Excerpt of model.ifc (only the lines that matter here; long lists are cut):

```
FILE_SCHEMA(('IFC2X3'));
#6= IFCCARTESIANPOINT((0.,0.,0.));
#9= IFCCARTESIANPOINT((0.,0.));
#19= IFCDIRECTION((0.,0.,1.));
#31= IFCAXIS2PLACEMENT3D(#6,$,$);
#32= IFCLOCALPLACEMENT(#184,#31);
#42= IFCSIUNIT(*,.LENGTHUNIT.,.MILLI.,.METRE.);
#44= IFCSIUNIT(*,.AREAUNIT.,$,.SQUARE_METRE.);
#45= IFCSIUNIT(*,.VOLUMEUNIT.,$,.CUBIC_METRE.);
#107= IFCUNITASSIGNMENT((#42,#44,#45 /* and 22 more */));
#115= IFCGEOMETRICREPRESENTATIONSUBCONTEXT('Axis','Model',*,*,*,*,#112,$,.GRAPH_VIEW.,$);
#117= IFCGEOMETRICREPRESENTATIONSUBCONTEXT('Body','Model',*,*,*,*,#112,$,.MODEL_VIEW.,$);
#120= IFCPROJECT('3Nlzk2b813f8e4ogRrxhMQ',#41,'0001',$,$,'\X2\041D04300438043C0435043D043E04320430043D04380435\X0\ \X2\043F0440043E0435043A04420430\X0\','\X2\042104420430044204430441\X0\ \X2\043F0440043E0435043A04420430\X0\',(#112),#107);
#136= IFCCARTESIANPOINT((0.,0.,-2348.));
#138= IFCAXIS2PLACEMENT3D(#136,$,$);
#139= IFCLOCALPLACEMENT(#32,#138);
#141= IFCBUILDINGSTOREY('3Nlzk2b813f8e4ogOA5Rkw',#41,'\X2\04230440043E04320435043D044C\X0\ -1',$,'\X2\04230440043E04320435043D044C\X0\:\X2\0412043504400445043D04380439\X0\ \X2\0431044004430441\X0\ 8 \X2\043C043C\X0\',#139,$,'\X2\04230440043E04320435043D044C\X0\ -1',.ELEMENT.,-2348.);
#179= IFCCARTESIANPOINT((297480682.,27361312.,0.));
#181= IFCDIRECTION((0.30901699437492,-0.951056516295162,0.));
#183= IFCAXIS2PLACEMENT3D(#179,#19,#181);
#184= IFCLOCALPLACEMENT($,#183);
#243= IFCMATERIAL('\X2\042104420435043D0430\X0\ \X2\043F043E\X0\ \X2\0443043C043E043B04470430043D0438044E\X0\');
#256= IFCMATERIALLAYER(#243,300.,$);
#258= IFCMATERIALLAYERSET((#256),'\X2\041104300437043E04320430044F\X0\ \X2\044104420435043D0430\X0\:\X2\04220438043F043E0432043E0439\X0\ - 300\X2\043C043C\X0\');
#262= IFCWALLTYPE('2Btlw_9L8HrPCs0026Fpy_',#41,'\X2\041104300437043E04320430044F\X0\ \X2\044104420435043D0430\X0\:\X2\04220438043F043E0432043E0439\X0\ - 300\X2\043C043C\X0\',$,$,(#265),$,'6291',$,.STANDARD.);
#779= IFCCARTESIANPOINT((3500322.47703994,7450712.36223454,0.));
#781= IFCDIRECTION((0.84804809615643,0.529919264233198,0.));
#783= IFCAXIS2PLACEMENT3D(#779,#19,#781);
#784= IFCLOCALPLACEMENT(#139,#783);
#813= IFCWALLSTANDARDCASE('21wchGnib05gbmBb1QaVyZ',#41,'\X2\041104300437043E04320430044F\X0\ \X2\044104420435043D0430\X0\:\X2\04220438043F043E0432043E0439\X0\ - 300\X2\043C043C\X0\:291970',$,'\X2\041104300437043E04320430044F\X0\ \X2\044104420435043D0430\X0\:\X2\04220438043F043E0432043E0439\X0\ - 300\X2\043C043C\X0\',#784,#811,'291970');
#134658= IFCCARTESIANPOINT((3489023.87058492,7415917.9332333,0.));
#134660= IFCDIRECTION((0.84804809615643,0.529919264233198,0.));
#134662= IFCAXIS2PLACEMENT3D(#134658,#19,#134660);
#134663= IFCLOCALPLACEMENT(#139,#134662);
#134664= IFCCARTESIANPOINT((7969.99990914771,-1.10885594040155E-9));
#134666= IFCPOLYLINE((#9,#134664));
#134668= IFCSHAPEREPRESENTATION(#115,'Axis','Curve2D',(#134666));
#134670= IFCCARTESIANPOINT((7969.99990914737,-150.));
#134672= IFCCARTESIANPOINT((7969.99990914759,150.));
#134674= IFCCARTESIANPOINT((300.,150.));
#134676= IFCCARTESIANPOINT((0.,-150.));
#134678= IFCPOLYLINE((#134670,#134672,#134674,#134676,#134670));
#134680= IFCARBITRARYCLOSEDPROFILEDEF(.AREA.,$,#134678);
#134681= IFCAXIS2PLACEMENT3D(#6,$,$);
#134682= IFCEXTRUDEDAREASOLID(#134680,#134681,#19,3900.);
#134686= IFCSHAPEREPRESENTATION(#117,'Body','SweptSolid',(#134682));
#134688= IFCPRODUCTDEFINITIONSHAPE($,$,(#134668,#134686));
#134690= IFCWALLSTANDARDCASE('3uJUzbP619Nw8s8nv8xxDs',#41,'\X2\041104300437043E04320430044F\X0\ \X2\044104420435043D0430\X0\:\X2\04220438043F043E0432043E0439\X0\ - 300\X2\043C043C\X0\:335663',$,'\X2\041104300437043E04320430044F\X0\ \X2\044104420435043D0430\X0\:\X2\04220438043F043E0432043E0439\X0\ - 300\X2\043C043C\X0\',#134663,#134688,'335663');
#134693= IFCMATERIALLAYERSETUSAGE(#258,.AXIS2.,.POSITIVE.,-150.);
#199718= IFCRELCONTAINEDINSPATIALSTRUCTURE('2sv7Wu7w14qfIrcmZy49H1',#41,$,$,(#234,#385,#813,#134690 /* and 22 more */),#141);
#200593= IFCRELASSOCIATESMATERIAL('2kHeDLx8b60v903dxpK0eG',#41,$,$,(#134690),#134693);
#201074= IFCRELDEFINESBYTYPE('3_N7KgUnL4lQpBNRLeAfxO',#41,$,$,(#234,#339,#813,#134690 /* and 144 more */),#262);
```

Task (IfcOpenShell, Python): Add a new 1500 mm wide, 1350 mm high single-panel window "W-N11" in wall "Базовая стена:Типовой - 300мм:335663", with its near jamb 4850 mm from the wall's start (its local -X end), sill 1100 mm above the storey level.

```python
import numpy as np
import ifcopenshell
import ifcopenshell.api.feature
import ifcopenshell.api.geometry
import ifcopenshell.api.root
import ifcopenshell.api.spatial
import ifcopenshell.api.type
import ifcopenshell.geom
import ifcopenshell.util.element
import ifcopenshell.util.placement
import ifcopenshell.util.representation
import ifcopenshell.util.shape
import ifcopenshell.util.unit

model = ifcopenshell.open("model.ifc")
unit_scale = ifcopenshell.util.unit.calculate_unit_scale(model)
settings = ifcopenshell.geom.settings()


def volume(element):
    """Net volume in cubic metres, openings subtracted."""
    shape = ifcopenshell.geom.create_shape(settings, element)
    return ifcopenshell.util.shape.get_volume(shape.geometry)


wall = model.by_guid("3uJUzbP619Nw8s8nv8xxDs")
storey = ifcopenshell.util.element.get_container(wall, ifc_class="IfcBuildingStorey")
context = ifcopenshell.util.representation.get_context(model, "Model", "Body", "MODEL_VIEW")
before = volume(wall)

width, height, from_end, sill = 1.5, 1.35, 4.85, 1.1  # metres

# The wall runs along its own X axis, and the end named is its -X end.
wall_shape = ifcopenshell.geom.create_shape(settings, wall)
x, y, z = ifcopenshell.util.shape.get_vertices(wall_shape.geometry).T
start = x.min() + from_end
face, thickness = float(y.min()), float(y.max() - y.min())
wall_matrix = ifcopenshell.util.placement.get_local_placement(wall.ObjectPlacement)
level = ifcopenshell.util.placement.get_local_placement(storey.ObjectPlacement)[2, 3]


def in_wall(x, y):
    """Placement at x, y metres in the wall's axes, at sill height."""
    matrix = wall_matrix.copy()
    matrix[:, 3] = wall_matrix @ np.array([x / unit_scale, y / unit_scale, 0.0, 1.0])
    matrix[2, 3] = level + sill / unit_scale
    return matrix


# Opening: a box that overshoots both wall faces by 50 mm.
opening = ifcopenshell.api.root.create_entity(model, ifc_class="IfcOpeningElement")
box = ifcopenshell.api.geometry.add_wall_representation(
    model, context=context, length=width, height=height, thickness=thickness + 0.1
)
ifcopenshell.api.geometry.assign_representation(model, product=opening, representation=box)
ifcopenshell.api.geometry.edit_object_placement(model, product=opening, matrix=in_wall(start, face - 0.05), is_si=False)
ifcopenshell.api.feature.add_feature(model, feature=opening, element=wall)

window = ifcopenshell.api.root.create_entity(model, ifc_class="IfcWindow", name="W-N11")
window.OverallWidth, window.OverallHeight = width / unit_scale, height / unit_scale
body = ifcopenshell.api.geometry.add_window_representation(
    model,
    context=context,
    overall_width=window.OverallWidth,
    overall_height=window.OverallHeight,
    partition_type="SINGLE_PANEL",
)
ifcopenshell.api.geometry.assign_representation(model, product=window, representation=body)
ifcopenshell.api.spatial.assign_container(model, products=[window], relating_structure=storey)
fills = ifcopenshell.api.feature.add_filling(model, opening=opening, element=window)
fills.OwnerHistory = window.OwnerHistory  # required in IFC2X3

# IFC2X3 keeps the operation on the window style.
style = ifcopenshell.api.root.create_entity(model, ifc_class="IfcWindowStyle", name="W-N11")
style.OperationType, style.ConstructionType = "SINGLE_PANEL", "NOTDEFINED"
style.ParameterTakesPrecedence = style.Sizeable = False
ifcopenshell.api.type.assign_type(model, related_objects=[window], relating_type=style)

# Centre the window in the wall's thickness.
ifcopenshell.api.geometry.edit_object_placement(model, product=window, matrix=in_wall(start, face), is_si=False)
window_shape = ifcopenshell.geom.create_shape(settings, window)
depth = ifcopenshell.util.shape.get_vertices(window_shape.geometry)[:, 1]
offset = face + thickness / 2 - (depth.min() + depth.max()) / 2
ifcopenshell.api.geometry.edit_object_placement(model, product=window, matrix=in_wall(start, offset), is_si=False)

after = volume(wall)

print(f"wall volume {before:.3f} -> {after:.3f} m3")

model.write("model-out.ifc")
```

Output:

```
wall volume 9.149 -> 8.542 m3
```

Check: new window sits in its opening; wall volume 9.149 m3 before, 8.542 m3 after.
